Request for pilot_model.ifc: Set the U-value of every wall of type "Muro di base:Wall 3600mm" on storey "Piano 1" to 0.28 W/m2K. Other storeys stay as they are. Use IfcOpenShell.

First a look at what the model holds.

```python
import ifcopenshell
import ifcopenshell.util.element

model = ifcopenshell.open("pilot_model.ifc")
print(model.schema)
storey = next(s for s in model.by_type("IfcBuildingStorey") if s.Name == "Piano 1")
walls = [e for e in ifcopenshell.util.element.get_decomposition(storey) if e.is_a("IfcWall")]
seen = {}
for e in walls:
    element_type = ifcopenshell.util.element.get_type(e)
    key = (element_type.Name if element_type != e and element_type else None, ifcopenshell.util.element.get_pset(e, "Pset_WallCommon", "ThermalTransmittance"))
    seen[key] = seen.get(key, 0) + 1
for (name, value), count in sorted(seen.items(), key=str):
    print(count, "x", name, "|", value)
```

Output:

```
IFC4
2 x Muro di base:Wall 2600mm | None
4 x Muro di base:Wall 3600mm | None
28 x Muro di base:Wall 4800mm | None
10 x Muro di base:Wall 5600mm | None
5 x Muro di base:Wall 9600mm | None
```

```python
import ifcopenshell
import ifcopenshell.api.pset
import ifcopenshell.util.element

model = ifcopenshell.open("pilot_model.ifc")

storey = next(s for s in model.by_type("IfcBuildingStorey") if s.Name == "Piano 1")
walls = [e for e in ifcopenshell.util.element.get_decomposition(storey) if e.is_a("IfcWall")]

count = 0
for e in walls:
    element_type = ifcopenshell.util.element.get_type(e)
    if element_type in (None, e) or element_type.Name != "Muro di base:Wall 3600mm":
        continue
    # add_pset returns the element's existing set when there is one.
    pset = ifcopenshell.api.pset.add_pset(model, product=e, name="Pset_WallCommon")
    ifcopenshell.api.pset.edit_pset(model, pset=pset, properties={"ThermalTransmittance": 0.28})
    count += 1

print(count, "walls updated")

model.write("pilot_model_v2.ifc")
```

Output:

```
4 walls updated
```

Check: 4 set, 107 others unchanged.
